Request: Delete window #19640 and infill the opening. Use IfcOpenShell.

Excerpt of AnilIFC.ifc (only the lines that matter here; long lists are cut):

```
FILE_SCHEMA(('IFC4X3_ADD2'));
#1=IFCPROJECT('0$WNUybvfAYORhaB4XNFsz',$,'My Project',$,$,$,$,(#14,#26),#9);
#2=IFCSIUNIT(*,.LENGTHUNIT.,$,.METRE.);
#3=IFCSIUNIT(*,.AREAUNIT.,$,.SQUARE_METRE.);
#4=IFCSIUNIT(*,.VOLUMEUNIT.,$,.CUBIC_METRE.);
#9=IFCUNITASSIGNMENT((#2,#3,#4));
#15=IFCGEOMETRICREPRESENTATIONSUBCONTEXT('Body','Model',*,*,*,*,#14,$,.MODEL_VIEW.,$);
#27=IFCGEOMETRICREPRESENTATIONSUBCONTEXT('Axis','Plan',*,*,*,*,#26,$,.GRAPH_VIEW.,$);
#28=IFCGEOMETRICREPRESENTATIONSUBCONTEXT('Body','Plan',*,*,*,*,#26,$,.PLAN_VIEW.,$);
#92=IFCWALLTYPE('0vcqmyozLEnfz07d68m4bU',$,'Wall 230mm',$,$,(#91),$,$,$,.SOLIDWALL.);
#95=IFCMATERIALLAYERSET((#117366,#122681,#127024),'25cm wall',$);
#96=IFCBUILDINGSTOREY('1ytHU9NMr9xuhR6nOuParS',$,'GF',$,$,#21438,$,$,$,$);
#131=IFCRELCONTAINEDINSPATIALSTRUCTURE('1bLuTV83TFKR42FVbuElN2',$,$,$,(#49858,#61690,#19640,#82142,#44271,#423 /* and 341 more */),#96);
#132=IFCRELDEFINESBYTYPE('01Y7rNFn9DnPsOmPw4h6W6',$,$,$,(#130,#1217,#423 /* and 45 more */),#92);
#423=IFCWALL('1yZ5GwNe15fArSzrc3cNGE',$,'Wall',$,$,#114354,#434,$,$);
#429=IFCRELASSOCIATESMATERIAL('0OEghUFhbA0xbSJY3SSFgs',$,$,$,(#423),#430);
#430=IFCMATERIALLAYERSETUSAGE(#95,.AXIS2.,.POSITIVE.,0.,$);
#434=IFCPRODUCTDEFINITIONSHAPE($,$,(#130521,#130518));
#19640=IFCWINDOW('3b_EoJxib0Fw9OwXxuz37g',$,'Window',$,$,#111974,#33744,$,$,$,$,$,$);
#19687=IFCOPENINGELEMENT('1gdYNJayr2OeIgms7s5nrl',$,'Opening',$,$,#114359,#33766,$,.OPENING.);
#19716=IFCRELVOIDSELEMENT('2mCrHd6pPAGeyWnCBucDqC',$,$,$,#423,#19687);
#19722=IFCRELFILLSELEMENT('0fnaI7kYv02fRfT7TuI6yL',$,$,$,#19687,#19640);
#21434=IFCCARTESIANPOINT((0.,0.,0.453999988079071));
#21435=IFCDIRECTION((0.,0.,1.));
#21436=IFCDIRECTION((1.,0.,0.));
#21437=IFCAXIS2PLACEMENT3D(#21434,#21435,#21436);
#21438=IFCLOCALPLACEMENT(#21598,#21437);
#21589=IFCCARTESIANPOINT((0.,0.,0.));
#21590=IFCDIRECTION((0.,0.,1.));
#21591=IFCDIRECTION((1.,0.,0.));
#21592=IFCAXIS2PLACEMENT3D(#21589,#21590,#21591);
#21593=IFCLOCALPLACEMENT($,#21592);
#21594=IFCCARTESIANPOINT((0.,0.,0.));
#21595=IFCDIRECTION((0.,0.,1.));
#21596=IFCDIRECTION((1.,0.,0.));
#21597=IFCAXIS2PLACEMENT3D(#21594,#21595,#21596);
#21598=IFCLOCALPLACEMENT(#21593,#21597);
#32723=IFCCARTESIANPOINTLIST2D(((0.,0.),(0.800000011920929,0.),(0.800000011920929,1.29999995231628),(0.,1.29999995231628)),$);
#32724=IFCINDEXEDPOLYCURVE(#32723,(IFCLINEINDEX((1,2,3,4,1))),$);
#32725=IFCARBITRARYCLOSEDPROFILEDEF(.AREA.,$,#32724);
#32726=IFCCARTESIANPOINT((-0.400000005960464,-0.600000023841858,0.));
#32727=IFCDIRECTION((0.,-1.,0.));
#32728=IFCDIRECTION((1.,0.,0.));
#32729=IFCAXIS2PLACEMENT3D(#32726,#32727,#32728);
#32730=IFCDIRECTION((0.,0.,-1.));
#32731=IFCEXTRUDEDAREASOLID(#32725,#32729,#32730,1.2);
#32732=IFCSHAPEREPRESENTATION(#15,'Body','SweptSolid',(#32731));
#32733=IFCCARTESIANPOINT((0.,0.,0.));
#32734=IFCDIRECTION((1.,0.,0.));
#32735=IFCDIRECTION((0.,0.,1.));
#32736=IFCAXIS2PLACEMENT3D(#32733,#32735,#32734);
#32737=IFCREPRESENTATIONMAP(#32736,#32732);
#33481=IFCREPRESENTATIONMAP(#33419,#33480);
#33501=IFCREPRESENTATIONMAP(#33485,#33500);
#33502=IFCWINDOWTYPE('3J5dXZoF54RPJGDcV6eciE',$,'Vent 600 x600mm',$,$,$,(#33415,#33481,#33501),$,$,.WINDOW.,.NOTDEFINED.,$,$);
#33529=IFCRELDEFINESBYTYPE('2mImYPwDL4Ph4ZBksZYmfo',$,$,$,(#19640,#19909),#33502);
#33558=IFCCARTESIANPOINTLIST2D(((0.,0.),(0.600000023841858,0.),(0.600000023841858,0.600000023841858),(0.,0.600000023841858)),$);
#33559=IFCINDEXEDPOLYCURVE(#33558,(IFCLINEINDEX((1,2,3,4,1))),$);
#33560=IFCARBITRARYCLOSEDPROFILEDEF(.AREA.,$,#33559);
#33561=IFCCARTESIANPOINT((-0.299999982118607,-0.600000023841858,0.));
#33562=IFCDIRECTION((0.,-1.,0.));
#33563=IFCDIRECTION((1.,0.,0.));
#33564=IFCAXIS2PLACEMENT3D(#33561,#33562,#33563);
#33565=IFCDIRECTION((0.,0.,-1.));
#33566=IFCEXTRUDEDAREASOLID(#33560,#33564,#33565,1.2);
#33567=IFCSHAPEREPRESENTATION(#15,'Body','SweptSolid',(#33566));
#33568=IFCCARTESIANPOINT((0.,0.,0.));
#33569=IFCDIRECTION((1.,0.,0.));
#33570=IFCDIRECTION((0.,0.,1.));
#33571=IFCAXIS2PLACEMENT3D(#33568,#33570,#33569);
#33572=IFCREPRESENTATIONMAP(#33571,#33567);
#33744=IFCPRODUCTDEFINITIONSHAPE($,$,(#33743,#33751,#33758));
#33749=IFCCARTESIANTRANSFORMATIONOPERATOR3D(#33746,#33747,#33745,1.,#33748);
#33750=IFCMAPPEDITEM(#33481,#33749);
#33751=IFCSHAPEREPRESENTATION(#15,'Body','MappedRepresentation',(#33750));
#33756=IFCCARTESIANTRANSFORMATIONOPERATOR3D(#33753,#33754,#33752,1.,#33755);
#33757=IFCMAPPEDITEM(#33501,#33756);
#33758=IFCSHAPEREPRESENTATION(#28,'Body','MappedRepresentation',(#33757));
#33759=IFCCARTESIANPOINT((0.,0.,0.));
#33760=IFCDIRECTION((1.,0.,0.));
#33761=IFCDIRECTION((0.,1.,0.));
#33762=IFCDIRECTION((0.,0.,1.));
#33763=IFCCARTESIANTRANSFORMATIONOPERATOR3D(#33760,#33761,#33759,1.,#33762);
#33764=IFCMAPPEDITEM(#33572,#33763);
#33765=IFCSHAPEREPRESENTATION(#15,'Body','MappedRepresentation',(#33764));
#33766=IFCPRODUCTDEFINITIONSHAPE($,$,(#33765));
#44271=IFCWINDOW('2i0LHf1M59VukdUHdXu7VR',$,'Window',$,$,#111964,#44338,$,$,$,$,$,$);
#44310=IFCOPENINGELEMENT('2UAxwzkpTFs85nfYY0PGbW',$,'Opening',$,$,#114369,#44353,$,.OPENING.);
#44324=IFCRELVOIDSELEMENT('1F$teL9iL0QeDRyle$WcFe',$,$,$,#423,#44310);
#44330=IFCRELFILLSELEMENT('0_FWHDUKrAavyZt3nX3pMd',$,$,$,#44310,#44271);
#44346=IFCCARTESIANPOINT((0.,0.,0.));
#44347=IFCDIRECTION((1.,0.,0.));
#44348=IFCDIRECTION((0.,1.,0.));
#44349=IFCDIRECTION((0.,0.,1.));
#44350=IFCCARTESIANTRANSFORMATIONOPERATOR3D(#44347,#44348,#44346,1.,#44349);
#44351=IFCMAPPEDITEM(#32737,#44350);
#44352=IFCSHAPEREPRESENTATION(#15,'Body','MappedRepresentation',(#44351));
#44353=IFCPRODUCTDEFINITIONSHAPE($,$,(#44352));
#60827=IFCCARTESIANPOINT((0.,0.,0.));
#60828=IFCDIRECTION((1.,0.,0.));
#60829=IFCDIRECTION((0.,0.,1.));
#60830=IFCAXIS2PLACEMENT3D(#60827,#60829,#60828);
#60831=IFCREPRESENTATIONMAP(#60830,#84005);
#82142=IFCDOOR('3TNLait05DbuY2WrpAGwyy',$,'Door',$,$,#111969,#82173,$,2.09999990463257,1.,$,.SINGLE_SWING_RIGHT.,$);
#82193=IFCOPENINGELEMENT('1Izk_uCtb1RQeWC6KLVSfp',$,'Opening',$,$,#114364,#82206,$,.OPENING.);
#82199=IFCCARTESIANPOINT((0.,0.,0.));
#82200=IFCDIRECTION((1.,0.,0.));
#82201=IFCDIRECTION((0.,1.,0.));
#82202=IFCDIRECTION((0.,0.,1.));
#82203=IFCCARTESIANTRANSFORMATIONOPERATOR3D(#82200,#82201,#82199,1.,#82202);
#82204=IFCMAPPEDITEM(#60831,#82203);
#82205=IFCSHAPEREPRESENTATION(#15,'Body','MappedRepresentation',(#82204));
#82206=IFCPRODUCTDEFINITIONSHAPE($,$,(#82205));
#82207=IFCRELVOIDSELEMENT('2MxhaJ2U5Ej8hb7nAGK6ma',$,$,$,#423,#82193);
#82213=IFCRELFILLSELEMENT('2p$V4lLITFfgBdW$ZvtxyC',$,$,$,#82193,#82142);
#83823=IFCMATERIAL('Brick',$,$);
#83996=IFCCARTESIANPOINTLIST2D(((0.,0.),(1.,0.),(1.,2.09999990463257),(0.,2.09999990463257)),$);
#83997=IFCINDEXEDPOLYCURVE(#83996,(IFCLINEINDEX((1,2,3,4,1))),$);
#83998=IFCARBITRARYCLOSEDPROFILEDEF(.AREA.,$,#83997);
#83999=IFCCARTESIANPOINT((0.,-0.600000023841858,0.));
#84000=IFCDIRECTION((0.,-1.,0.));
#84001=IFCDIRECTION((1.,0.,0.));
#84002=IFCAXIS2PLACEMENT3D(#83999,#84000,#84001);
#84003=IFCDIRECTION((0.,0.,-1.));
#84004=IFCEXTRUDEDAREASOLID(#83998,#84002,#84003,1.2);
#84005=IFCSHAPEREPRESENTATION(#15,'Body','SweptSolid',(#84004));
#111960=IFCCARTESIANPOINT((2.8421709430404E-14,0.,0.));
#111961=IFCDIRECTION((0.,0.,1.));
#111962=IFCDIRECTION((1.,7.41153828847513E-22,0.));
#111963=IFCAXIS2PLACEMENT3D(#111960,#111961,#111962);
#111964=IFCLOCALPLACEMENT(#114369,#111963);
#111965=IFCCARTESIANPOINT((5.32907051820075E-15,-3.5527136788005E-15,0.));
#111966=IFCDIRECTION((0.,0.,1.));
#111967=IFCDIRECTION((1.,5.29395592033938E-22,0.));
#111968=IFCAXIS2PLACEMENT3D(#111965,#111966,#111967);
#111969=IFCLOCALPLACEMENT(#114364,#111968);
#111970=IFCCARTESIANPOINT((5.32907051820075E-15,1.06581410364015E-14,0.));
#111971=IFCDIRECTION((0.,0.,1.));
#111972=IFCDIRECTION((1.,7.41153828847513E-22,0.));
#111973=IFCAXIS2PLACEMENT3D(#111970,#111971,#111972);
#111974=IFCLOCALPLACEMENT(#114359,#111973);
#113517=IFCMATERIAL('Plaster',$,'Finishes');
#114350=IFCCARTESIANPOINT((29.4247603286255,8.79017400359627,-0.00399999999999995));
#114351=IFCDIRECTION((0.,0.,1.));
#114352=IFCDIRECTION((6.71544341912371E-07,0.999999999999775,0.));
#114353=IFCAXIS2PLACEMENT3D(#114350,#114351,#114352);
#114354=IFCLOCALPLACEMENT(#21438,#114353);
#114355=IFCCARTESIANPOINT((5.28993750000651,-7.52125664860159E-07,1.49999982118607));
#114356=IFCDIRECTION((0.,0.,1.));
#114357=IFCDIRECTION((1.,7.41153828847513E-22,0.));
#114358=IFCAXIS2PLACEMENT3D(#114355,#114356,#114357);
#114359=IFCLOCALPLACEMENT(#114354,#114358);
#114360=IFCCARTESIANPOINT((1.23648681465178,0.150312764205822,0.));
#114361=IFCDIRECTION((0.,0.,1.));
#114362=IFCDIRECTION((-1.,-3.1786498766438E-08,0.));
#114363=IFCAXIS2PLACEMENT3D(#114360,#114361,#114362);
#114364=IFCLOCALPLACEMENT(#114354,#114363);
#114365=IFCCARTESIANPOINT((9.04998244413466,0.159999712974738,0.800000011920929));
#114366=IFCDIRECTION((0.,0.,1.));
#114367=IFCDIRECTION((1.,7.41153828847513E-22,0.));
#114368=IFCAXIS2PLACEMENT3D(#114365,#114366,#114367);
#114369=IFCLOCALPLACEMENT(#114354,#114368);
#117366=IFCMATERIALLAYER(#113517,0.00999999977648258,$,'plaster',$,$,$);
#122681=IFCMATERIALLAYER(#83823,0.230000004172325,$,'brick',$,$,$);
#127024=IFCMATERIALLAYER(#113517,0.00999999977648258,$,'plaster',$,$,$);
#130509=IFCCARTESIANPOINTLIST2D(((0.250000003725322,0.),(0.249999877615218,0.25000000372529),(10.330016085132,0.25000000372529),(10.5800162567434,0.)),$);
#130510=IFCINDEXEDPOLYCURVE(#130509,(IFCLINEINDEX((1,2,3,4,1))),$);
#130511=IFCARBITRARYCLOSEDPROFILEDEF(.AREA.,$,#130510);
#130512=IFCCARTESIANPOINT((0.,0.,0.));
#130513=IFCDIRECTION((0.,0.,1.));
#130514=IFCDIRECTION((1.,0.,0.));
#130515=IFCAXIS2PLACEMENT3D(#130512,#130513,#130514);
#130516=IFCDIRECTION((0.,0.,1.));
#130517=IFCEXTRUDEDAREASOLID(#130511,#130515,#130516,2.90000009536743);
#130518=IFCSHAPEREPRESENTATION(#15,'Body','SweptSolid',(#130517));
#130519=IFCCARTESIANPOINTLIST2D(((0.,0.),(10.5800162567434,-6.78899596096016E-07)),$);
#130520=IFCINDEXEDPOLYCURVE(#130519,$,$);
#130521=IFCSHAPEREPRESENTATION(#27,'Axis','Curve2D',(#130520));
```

```python
import ifcopenshell
import ifcopenshell.api.feature
import ifcopenshell.api.root
import ifcopenshell.geom
import ifcopenshell.util.shape

model = ifcopenshell.open("AnilIFC.ifc")
settings = ifcopenshell.geom.settings()


def volume(element):
    """Net volume in cubic metres, openings subtracted."""
    shape = ifcopenshell.geom.create_shape(settings, element)
    return ifcopenshell.util.shape.get_volume(shape.geometry)


window = model.by_id(19640)
opening = window.FillsVoids[0].RelatingOpeningElement
wall = opening.VoidsElements[0].RelatingBuildingElement
before = volume(wall)

ifcopenshell.api.root.remove_product(model, product=window)
ifcopenshell.api.feature.remove_feature(model, feature=opening)

after = volume(wall)

print(f"wall volume {before:.3f} -> {after:.3f} m3")

model.write("AnilIFC_v2.ifc")
```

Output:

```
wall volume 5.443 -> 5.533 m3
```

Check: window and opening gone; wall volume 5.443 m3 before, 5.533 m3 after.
